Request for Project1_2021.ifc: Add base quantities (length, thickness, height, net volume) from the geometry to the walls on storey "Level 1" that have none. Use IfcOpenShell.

First a look at what the model holds.

```python
import ifcopenshell
import ifcopenshell.util.element
import ifcopenshell.util.unit

model = ifcopenshell.open("Project1_2021.ifc")
print(model.schema)
for unit_type in ("LENGTHUNIT", "AREAUNIT", "VOLUMEUNIT"):
    print(unit_type, ifcopenshell.util.unit.calculate_unit_scale(model, unit_type))
storey = next(s for s in model.by_type("IfcBuildingStorey") if s.Name == "Level 1")
walls = [e for e in ifcopenshell.util.element.get_decomposition(storey) if e.is_a("IfcWall")]
for e in sorted(walls, key=lambda e: e.id()):
    print(e.id(), e.is_a(), e.Name, list(ifcopenshell.util.element.get_psets(e, qtos_only=True)), sep=" | ")
```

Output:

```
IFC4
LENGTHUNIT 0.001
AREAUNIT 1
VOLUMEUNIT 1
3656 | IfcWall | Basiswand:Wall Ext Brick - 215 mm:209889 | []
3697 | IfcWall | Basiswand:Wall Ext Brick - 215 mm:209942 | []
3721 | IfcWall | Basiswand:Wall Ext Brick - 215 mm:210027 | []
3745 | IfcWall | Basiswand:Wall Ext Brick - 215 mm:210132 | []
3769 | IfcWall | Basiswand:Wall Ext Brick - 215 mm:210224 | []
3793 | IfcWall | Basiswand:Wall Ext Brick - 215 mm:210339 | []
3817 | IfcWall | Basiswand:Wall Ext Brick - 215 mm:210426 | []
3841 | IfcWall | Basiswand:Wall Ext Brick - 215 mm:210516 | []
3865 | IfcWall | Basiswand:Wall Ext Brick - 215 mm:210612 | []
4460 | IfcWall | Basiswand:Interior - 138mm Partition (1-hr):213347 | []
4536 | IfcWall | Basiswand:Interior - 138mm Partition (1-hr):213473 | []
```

```python
import ifcopenshell
import ifcopenshell.api.pset
import ifcopenshell.geom
import ifcopenshell.util.element
import ifcopenshell.util.shape
import ifcopenshell.util.unit

model = ifcopenshell.open("Project1_2021.ifc")
unit_scale = ifcopenshell.util.unit.calculate_unit_scale(model)
volume_scale = ifcopenshell.util.unit.calculate_unit_scale(model, "VOLUMEUNIT")
settings = ifcopenshell.geom.settings()

storey = next(s for s in model.by_type("IfcBuildingStorey") if s.Name == "Level 1")
walls = [e for e in ifcopenshell.util.element.get_decomposition(storey) if e.is_a("IfcWall")]

for e in sorted(walls, key=lambda e: e.id()):
    if ifcopenshell.util.element.get_psets(e, qtos_only=True, should_inherit=False):
        continue
    # Geometry comes back in metres, in the element's own axes.
    shape = ifcopenshell.geom.create_shape(settings, e)
    values = {
        "Length": ifcopenshell.util.shape.get_x(shape.geometry) / unit_scale,
        "Width": ifcopenshell.util.shape.get_y(shape.geometry) / unit_scale,
        "Height": ifcopenshell.util.shape.get_z(shape.geometry) / unit_scale,
        "NetVolume": ifcopenshell.util.shape.get_volume(shape.geometry) / volume_scale,
    }
    qto = ifcopenshell.api.pset.add_qto(model, product=e, name="Qto_WallBaseQuantities")
    ifcopenshell.api.pset.edit_qto(model, qto=qto, properties=values)
    print(e.id(), {k: round(v, 3) for k, v in values.items()})

model.write("Project1_2021_updated.ifc")
```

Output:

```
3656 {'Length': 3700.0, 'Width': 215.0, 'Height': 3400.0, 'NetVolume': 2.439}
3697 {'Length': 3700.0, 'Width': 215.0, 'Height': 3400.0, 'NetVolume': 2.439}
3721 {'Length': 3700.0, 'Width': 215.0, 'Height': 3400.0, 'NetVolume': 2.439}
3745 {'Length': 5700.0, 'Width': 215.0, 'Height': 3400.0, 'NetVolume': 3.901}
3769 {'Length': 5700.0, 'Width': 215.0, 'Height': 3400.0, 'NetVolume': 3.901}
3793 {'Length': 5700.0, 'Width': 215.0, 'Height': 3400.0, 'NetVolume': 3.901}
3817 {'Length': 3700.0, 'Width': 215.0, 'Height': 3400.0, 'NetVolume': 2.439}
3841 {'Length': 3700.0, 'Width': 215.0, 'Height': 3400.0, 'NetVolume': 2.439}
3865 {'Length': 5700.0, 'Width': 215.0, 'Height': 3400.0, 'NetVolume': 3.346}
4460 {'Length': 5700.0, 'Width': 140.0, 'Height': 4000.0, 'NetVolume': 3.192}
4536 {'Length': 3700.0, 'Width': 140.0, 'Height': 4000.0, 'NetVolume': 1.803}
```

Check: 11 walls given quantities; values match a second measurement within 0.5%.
